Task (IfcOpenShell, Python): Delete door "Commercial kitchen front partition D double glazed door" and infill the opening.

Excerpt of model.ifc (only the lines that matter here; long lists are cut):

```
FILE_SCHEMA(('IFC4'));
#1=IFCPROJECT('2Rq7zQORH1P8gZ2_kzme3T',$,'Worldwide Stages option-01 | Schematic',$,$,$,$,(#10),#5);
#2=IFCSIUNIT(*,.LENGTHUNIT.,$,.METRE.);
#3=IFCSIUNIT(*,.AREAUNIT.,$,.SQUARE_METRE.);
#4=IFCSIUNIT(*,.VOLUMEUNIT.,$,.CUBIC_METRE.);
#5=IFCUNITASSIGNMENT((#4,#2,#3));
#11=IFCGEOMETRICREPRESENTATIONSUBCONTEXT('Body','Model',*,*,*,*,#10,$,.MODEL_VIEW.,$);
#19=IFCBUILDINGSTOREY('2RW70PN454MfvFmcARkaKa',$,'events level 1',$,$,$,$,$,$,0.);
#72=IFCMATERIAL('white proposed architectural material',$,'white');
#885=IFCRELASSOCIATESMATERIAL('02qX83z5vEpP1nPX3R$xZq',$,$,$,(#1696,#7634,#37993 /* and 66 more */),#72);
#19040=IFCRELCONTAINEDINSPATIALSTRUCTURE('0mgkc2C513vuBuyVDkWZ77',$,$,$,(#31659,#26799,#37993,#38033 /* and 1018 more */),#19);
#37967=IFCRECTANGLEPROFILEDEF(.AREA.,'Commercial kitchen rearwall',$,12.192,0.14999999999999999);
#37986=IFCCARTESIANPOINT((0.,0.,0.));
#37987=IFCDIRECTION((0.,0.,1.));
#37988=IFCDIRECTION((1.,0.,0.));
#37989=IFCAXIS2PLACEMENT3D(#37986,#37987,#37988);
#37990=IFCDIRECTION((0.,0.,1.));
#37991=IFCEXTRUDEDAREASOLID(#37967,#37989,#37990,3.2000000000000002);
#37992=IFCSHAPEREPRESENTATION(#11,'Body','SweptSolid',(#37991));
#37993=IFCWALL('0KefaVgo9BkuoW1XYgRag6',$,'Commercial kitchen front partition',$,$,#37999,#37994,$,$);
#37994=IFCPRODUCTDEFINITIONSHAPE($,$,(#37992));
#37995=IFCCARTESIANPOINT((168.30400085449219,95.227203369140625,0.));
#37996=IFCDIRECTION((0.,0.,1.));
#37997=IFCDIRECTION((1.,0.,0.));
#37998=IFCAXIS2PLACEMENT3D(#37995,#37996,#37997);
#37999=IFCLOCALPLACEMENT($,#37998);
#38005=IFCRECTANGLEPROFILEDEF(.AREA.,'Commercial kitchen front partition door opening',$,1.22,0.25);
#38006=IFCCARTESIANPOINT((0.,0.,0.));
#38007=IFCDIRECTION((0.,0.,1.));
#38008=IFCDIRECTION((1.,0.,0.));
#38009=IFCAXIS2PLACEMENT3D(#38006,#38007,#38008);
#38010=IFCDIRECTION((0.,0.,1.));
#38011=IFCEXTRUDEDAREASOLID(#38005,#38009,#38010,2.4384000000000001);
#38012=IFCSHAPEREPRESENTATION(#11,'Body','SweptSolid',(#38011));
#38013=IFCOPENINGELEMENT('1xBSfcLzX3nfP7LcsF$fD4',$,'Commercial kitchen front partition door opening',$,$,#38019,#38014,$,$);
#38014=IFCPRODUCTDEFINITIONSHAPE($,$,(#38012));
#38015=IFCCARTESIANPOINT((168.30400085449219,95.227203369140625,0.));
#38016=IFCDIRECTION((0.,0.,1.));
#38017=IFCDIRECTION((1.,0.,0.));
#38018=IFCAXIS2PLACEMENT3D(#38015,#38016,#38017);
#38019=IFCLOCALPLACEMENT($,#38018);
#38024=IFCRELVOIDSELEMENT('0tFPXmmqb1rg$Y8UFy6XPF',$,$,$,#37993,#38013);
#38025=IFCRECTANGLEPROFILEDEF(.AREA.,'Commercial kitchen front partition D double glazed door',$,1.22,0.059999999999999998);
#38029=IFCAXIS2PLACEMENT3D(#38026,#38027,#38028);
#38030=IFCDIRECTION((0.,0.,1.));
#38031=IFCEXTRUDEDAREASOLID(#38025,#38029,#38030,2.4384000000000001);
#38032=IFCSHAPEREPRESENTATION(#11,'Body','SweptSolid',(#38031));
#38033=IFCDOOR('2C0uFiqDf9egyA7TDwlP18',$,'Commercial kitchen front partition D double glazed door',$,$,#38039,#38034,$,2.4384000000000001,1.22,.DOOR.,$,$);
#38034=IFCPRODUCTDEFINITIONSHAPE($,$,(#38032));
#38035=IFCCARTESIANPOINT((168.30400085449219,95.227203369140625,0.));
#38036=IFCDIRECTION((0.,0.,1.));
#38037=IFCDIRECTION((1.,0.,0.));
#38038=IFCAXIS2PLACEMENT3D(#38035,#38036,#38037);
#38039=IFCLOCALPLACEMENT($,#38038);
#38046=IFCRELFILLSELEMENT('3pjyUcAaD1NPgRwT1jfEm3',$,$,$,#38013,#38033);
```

```python
import ifcopenshell
import ifcopenshell.api.feature
import ifcopenshell.api.root
import ifcopenshell.geom
import ifcopenshell.util.shape

model = ifcopenshell.open("model.ifc")
settings = ifcopenshell.geom.settings()


def volume(element):
    """Net volume in cubic metres, openings subtracted."""
    shape = ifcopenshell.geom.create_shape(settings, element)
    return ifcopenshell.util.shape.get_volume(shape.geometry)


door = model.by_guid("2C0uFiqDf9egyA7TDwlP18")
opening = door.FillsVoids[0].RelatingOpeningElement
wall = opening.VoidsElements[0].RelatingBuildingElement
before = volume(wall)

ifcopenshell.api.root.remove_product(model, product=door)
ifcopenshell.api.feature.remove_feature(model, feature=opening)

after = volume(wall)

print(f"wall volume {before:.3f} -> {after:.3f} m3")

model.write("model_edited.ifc")
```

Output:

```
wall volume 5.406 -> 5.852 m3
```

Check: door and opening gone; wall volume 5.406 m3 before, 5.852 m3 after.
